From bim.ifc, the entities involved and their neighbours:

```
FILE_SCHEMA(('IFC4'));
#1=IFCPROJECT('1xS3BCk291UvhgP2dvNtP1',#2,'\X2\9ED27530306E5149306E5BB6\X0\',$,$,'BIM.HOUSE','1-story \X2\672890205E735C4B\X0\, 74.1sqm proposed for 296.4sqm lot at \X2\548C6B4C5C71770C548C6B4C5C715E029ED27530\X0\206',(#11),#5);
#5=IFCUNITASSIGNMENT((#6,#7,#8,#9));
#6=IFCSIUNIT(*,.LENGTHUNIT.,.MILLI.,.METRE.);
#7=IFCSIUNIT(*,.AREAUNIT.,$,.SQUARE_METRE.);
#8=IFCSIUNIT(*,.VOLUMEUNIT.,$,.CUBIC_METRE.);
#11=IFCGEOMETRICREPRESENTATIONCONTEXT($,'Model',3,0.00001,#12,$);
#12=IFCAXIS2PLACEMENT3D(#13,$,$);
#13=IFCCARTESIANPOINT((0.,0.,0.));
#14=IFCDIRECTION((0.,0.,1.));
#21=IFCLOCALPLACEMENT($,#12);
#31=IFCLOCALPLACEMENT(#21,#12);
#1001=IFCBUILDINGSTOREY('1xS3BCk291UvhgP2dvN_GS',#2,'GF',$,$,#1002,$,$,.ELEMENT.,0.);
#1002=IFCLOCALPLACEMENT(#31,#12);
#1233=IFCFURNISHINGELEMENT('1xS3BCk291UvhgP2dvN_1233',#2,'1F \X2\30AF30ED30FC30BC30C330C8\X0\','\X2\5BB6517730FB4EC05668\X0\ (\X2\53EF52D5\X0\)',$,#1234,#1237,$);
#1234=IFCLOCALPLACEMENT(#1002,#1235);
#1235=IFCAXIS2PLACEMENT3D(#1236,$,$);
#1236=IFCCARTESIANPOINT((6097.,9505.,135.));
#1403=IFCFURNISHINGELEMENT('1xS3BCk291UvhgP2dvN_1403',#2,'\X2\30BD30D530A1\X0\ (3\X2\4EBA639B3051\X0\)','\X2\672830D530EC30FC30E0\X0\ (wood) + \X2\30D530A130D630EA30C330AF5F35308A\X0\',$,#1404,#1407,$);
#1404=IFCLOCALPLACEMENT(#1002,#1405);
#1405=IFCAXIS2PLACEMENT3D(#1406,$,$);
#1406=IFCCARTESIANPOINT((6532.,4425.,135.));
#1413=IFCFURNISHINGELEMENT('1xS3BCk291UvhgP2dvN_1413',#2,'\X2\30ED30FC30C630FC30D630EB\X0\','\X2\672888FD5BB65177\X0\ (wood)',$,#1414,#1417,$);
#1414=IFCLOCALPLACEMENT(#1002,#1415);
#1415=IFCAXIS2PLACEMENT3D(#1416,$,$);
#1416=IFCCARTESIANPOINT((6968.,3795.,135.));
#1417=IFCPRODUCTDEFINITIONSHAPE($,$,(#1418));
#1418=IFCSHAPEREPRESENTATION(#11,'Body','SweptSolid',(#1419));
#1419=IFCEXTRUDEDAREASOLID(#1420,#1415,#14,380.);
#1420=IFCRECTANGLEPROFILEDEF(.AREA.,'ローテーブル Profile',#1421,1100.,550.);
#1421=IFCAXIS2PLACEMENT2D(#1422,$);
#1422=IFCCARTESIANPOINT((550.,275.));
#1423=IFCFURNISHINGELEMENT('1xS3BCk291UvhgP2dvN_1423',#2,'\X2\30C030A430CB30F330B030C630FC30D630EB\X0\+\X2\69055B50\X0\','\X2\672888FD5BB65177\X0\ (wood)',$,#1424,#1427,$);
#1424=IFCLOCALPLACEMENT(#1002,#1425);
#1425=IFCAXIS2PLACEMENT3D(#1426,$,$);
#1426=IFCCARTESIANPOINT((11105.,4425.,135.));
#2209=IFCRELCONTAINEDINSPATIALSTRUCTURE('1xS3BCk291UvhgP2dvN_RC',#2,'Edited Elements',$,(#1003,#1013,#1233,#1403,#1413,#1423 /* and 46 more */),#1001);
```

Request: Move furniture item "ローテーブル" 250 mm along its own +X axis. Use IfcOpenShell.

```python
import ifcopenshell
import ifcopenshell.api.geometry
import ifcopenshell.util.placement

model = ifcopenshell.open("bim.ifc")

item = model.by_id(1413)
matrix = ifcopenshell.util.placement.get_local_placement(item.ObjectPlacement)
matrix[:3, 3] += matrix[:3, 0] * 250.0
ifcopenshell.api.geometry.edit_object_placement(model, product=item, matrix=matrix, is_si=False)

print(ifcopenshell.util.placement.get_local_placement(item.ObjectPlacement).round(3) + 0.0)

model.write("bim-out.ifc")
```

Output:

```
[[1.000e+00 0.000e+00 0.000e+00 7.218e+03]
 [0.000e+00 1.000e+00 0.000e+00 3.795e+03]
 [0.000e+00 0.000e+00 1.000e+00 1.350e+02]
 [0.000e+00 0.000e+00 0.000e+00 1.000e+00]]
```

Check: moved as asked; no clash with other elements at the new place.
